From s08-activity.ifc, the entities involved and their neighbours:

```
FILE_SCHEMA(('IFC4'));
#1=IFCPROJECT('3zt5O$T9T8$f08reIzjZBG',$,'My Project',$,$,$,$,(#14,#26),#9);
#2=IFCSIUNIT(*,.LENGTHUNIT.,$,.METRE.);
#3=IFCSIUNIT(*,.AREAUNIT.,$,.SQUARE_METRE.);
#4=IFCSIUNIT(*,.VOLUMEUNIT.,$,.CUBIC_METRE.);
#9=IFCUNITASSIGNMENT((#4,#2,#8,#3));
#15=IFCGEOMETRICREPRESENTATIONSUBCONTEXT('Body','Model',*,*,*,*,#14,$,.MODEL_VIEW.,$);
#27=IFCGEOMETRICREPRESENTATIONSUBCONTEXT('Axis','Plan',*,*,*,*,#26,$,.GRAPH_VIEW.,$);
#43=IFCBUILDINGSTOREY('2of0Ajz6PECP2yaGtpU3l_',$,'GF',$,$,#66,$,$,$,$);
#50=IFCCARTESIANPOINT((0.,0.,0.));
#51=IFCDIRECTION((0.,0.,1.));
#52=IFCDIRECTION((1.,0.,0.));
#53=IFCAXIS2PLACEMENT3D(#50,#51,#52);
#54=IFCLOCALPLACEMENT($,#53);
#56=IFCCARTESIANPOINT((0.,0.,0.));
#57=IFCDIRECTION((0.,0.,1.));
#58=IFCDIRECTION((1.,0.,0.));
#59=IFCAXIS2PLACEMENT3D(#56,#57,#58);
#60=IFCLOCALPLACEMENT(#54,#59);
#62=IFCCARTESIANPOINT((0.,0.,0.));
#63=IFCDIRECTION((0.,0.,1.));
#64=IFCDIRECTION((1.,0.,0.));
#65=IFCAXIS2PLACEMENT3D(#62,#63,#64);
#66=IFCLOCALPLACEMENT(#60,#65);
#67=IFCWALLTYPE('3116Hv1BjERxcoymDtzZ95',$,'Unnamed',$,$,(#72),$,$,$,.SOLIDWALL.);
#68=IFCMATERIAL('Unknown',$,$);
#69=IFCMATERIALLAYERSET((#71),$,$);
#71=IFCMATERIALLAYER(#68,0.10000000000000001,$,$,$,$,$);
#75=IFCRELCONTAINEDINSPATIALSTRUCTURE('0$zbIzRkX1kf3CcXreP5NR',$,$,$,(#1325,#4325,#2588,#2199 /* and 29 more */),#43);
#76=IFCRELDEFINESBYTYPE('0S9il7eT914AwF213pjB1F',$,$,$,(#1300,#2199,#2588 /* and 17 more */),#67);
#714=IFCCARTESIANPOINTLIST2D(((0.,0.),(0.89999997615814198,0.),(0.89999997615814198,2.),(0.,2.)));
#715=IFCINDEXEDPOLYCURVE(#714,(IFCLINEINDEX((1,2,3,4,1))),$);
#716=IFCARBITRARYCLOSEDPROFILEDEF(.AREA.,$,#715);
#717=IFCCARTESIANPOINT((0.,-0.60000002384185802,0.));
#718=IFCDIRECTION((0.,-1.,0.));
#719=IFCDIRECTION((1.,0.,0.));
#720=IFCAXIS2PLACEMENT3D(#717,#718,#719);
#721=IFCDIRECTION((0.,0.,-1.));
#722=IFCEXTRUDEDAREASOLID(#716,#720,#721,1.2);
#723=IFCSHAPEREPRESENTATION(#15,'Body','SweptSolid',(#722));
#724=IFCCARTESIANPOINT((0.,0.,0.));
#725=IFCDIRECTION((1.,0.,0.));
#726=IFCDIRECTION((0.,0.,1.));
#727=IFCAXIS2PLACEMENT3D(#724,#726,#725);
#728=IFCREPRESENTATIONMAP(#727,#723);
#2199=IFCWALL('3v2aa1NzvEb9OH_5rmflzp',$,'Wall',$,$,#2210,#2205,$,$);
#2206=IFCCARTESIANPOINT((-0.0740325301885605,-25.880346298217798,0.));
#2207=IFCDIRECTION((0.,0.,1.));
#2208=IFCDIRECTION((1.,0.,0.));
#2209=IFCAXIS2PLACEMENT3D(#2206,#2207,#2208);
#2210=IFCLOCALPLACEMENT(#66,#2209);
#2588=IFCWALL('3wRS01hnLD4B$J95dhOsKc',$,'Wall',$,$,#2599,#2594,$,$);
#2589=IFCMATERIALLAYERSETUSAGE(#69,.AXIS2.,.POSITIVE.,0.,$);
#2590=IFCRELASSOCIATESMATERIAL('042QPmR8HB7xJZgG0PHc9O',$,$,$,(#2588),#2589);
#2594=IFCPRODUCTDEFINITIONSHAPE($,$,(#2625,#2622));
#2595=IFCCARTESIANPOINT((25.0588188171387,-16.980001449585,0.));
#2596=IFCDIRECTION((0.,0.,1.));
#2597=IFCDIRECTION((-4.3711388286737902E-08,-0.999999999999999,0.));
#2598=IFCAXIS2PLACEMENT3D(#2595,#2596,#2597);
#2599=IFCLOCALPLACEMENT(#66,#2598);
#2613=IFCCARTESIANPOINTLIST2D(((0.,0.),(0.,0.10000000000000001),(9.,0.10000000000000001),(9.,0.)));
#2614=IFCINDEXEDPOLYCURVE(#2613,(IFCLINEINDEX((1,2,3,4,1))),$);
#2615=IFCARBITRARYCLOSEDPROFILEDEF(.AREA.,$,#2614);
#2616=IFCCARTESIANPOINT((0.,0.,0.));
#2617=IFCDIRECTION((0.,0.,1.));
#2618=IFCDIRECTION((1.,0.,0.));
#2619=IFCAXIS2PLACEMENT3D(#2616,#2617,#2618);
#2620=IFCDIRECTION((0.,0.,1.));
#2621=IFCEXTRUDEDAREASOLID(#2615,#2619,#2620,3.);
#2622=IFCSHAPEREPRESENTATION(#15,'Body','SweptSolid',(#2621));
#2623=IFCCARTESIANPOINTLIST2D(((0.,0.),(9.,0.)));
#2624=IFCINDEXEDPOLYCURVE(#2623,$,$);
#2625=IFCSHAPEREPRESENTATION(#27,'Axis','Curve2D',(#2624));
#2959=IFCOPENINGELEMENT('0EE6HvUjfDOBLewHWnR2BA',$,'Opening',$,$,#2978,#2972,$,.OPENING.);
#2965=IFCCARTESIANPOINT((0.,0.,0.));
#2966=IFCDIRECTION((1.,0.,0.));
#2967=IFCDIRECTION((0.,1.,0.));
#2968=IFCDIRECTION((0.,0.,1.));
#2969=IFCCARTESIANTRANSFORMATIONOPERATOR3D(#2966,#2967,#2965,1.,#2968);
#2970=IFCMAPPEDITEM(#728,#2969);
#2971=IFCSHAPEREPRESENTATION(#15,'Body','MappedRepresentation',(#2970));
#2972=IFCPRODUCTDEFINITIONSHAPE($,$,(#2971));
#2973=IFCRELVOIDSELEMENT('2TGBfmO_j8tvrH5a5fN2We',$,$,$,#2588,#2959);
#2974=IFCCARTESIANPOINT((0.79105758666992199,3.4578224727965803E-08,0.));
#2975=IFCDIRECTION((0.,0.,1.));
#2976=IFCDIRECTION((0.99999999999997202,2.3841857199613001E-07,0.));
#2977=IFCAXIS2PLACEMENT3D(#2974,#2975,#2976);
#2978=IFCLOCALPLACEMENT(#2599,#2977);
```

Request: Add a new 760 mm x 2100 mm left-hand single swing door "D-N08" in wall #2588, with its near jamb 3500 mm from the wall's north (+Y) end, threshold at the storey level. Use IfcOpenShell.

```python
import numpy as np
import ifcopenshell
import ifcopenshell.api.feature
import ifcopenshell.api.geometry
import ifcopenshell.api.root
import ifcopenshell.api.spatial
import ifcopenshell.geom
import ifcopenshell.util.element
import ifcopenshell.util.placement
import ifcopenshell.util.representation
import ifcopenshell.util.shape
import ifcopenshell.util.unit

model = ifcopenshell.open("s08-activity.ifc")
unit_scale = ifcopenshell.util.unit.calculate_unit_scale(model)
settings = ifcopenshell.geom.settings()


def volume(element):
    """Net volume in cubic metres, openings subtracted."""
    shape = ifcopenshell.geom.create_shape(settings, element)
    return ifcopenshell.util.shape.get_volume(shape.geometry)


wall = model.by_id(2588)
storey = ifcopenshell.util.element.get_container(wall, ifc_class="IfcBuildingStorey")
context = ifcopenshell.util.representation.get_context(model, "Model", "Body", "MODEL_VIEW")
before = volume(wall)

width, height, from_end, sill = 0.76, 2.1, 3.5, 0.0  # metres

# The wall runs along its own X axis, and the end named is its -X end.
wall_shape = ifcopenshell.geom.create_shape(settings, wall)
x, y, z = ifcopenshell.util.shape.get_vertices(wall_shape.geometry).T
start = x.min() + from_end
face, thickness = float(y.min()), float(y.max() - y.min())
wall_matrix = ifcopenshell.util.placement.get_local_placement(wall.ObjectPlacement)
level = ifcopenshell.util.placement.get_local_placement(storey.ObjectPlacement)[2, 3]


def in_wall(x, y):
    """Placement at x, y metres in the wall's axes, at sill height."""
    matrix = wall_matrix.copy()
    matrix[:, 3] = wall_matrix @ np.array([x / unit_scale, y / unit_scale, 0.0, 1.0])
    matrix[2, 3] = level + sill / unit_scale
    return matrix


# Opening: a box that overshoots both wall faces by 50 mm.
opening = ifcopenshell.api.root.create_entity(model, ifc_class="IfcOpeningElement", predefined_type="OPENING")
box = ifcopenshell.api.geometry.add_wall_representation(
    model, context=context, length=width, height=height, thickness=thickness + 0.1
)
ifcopenshell.api.geometry.assign_representation(model, product=opening, representation=box)
ifcopenshell.api.geometry.edit_object_placement(model, product=opening, matrix=in_wall(start, face - 0.05), is_si=False)
ifcopenshell.api.feature.add_feature(model, feature=opening, element=wall)

door = ifcopenshell.api.root.create_entity(model, ifc_class="IfcDoor", name="D-N08", predefined_type="DOOR")
door.OverallWidth, door.OverallHeight = width / unit_scale, height / unit_scale
door.OperationType = "SINGLE_SWING_LEFT"
body = ifcopenshell.api.geometry.add_door_representation(
    model,
    context=context,
    overall_width=door.OverallWidth,
    overall_height=door.OverallHeight,
    operation_type="SINGLE_SWING_LEFT",
    lining_properties={"LiningDepth": thickness / unit_scale, "ThresholdDepth": thickness / unit_scale},
)
ifcopenshell.api.geometry.assign_representation(model, product=door, representation=body)
ifcopenshell.api.spatial.assign_container(model, products=[door], relating_structure=storey)
ifcopenshell.api.feature.add_filling(model, opening=opening, element=door)

# The lining spans the wall, so the door starts at the wall face.
ifcopenshell.api.geometry.edit_object_placement(model, product=door, matrix=in_wall(start, face), is_si=False)

after = volume(wall)

print(f"wall volume {before:.3f} -> {after:.3f} m3")

model.write("s08-activity-out.ifc")
```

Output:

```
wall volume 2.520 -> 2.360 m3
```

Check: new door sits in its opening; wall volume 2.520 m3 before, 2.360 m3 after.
